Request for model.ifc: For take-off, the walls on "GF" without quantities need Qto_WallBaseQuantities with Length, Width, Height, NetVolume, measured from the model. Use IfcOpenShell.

First a look at what the model holds.

```python
import ifcopenshell
import ifcopenshell.util.element
import ifcopenshell.util.unit

model = ifcopenshell.open("model.ifc")
print(model.schema)
for unit_type in ("LENGTHUNIT", "AREAUNIT", "VOLUMEUNIT"):
    print(unit_type, ifcopenshell.util.unit.calculate_unit_scale(model, unit_type))
storey = next(s for s in model.by_type("IfcBuildingStorey") if s.Name == "GF")
walls = [e for e in ifcopenshell.util.element.get_decomposition(storey) if e.is_a("IfcWall")]
for e in sorted(walls, key=lambda e: e.id()):
    print(e.id(), e.is_a(), e.Name, list(ifcopenshell.util.element.get_psets(e, qtos_only=True)), sep=" | ")
```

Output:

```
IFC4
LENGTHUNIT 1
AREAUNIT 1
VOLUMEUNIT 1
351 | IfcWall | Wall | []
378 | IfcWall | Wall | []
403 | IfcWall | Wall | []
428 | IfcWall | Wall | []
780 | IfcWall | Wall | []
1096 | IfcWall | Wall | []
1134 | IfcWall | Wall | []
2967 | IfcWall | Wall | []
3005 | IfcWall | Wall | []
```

```python
import ifcopenshell
import ifcopenshell.api.pset
import ifcopenshell.geom
import ifcopenshell.util.element
import ifcopenshell.util.shape
import ifcopenshell.util.unit

model = ifcopenshell.open("model.ifc")
unit_scale = ifcopenshell.util.unit.calculate_unit_scale(model)
volume_scale = ifcopenshell.util.unit.calculate_unit_scale(model, "VOLUMEUNIT")
settings = ifcopenshell.geom.settings()

storey = next(s for s in model.by_type("IfcBuildingStorey") if s.Name == "GF")
walls = [e for e in ifcopenshell.util.element.get_decomposition(storey) if e.is_a("IfcWall")]

for e in sorted(walls, key=lambda e: e.id()):
    if ifcopenshell.util.element.get_psets(e, qtos_only=True, should_inherit=False):
        continue
    # Geometry comes back in metres, in the element's own axes.
    shape = ifcopenshell.geom.create_shape(settings, e)
    values = {
        "Length": ifcopenshell.util.shape.get_x(shape.geometry) / unit_scale,
        "Width": ifcopenshell.util.shape.get_y(shape.geometry) / unit_scale,
        "Height": ifcopenshell.util.shape.get_z(shape.geometry) / unit_scale,
        "NetVolume": ifcopenshell.util.shape.get_volume(shape.geometry) / volume_scale,
    }
    qto = ifcopenshell.api.pset.add_qto(model, product=e, name="Qto_WallBaseQuantities")
    ifcopenshell.api.pset.edit_qto(model, qto=qto, properties=values)
    print(e.id(), {k: round(v, 3) for k, v in values.items()})

model.write("model_updated.ifc")
```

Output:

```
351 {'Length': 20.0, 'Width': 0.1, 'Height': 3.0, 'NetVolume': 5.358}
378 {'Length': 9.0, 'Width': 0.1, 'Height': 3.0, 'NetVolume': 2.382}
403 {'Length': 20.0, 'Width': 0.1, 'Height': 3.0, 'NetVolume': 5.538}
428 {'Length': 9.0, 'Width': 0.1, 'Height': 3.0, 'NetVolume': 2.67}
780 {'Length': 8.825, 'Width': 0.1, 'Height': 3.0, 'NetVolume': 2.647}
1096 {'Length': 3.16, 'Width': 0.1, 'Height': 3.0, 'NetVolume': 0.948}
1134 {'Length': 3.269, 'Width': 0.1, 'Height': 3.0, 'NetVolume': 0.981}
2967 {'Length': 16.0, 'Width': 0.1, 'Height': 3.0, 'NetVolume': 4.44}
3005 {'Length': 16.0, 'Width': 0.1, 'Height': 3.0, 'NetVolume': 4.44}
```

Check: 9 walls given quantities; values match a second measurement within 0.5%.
